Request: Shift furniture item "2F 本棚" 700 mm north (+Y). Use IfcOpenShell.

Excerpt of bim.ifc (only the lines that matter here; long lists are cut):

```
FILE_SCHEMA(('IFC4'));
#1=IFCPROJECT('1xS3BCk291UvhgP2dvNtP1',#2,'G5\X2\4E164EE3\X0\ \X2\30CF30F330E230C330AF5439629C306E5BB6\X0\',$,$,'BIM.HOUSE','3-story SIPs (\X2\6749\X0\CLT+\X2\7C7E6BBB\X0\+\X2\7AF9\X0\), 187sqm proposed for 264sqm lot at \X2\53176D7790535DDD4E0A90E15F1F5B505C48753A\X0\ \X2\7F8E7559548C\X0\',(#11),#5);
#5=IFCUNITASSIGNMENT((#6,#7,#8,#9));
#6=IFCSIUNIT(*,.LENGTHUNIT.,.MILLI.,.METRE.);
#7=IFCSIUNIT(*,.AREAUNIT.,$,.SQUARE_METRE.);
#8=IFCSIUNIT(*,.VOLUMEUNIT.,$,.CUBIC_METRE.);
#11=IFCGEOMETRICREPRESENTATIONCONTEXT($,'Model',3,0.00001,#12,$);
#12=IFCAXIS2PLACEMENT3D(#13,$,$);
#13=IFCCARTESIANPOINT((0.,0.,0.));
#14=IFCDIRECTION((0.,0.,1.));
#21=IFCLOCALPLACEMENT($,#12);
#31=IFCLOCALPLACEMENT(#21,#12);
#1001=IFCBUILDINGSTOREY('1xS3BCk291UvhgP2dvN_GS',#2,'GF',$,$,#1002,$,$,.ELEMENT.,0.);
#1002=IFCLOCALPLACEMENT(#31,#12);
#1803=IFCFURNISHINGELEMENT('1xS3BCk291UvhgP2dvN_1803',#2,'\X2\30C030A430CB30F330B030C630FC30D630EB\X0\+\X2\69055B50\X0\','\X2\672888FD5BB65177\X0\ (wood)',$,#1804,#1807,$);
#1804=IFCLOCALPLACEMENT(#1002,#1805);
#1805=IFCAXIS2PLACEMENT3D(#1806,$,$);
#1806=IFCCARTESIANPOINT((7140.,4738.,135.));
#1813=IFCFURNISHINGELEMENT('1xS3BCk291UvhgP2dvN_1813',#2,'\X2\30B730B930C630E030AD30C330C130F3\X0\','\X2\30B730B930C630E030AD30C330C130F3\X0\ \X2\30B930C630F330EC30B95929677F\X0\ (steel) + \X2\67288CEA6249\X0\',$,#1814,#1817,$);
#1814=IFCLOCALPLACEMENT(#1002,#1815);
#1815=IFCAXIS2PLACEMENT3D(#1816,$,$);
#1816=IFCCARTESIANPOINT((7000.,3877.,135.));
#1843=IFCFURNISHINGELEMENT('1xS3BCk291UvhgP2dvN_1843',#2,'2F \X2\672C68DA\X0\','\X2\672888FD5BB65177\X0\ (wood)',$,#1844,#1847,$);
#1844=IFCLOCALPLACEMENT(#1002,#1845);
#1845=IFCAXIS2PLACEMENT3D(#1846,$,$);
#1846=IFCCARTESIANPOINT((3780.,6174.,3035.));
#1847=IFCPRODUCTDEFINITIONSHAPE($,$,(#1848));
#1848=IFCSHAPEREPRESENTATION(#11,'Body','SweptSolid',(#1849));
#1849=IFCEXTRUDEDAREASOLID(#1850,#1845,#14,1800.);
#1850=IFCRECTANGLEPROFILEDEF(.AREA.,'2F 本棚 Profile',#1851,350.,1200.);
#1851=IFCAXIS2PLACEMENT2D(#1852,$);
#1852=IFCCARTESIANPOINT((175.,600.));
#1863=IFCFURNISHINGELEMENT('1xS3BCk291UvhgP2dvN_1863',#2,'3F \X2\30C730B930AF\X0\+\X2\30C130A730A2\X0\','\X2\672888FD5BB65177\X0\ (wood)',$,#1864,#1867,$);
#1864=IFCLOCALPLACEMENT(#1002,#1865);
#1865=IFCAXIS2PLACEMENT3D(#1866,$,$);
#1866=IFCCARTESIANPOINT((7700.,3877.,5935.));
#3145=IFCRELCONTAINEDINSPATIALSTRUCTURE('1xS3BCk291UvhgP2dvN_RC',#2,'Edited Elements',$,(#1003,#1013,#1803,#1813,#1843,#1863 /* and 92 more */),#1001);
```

```python
import ifcopenshell
import ifcopenshell.api.geometry
import ifcopenshell.util.placement
import ifcopenshell.util.unit

model = ifcopenshell.open("bim.ifc")
unit_scale = ifcopenshell.util.unit.calculate_unit_scale(model)

item = model.by_guid("1xS3BCk291UvhgP2dvN_1843")
matrix = ifcopenshell.util.placement.get_local_placement(item.ObjectPlacement)
matrix[1, 3] += 0.7 / unit_scale
ifcopenshell.api.geometry.edit_object_placement(model, product=item, matrix=matrix, is_si=False)

print(ifcopenshell.util.placement.get_local_placement(item.ObjectPlacement).round(3) + 0.0)

model.write("bim_rev.ifc")
```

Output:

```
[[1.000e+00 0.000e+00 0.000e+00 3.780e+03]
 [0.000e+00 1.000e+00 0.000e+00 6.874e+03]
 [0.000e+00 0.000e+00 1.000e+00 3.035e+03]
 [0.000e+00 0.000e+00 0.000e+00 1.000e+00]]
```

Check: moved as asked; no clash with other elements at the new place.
